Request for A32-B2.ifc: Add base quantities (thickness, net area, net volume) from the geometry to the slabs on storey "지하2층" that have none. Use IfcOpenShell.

First a look at what the model holds.

```python
import ifcopenshell
import ifcopenshell.util.element
import ifcopenshell.util.unit

model = ifcopenshell.open("A32-B2.ifc")
print(model.schema)
for unit_type in ("LENGTHUNIT", "AREAUNIT", "VOLUMEUNIT"):
    print(unit_type, ifcopenshell.util.unit.calculate_unit_scale(model, unit_type))
storey = next(s for s in model.by_type("IfcBuildingStorey") if s.Name == "지하2층")
slabs = [e for e in ifcopenshell.util.element.get_decomposition(storey) if e.is_a("IfcSlab")]
for e in sorted(slabs, key=lambda e: e.id()):
    print(e.id(), e.is_a(), e.Name, list(ifcopenshell.util.element.get_psets(e, qtos_only=True)), sep=" | ")
```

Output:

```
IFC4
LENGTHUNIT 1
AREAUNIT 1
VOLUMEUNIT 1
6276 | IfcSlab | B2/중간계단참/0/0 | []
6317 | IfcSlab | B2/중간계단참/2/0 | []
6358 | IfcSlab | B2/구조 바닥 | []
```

```python
import ifcopenshell
import ifcopenshell.api.pset
import ifcopenshell.geom
import ifcopenshell.util.element
import ifcopenshell.util.shape
import ifcopenshell.util.unit

model = ifcopenshell.open("A32-B2.ifc")
unit_scale = ifcopenshell.util.unit.calculate_unit_scale(model)
area_scale = ifcopenshell.util.unit.calculate_unit_scale(model, "AREAUNIT")
volume_scale = ifcopenshell.util.unit.calculate_unit_scale(model, "VOLUMEUNIT")
settings = ifcopenshell.geom.settings()

storey = next(s for s in model.by_type("IfcBuildingStorey") if s.Name == "지하2층")
slabs = [e for e in ifcopenshell.util.element.get_decomposition(storey) if e.is_a("IfcSlab")]

for e in sorted(slabs, key=lambda e: e.id()):
    if ifcopenshell.util.element.get_psets(e, qtos_only=True, should_inherit=False):
        continue
    # Geometry comes back in metres, in the element's own axes.
    shape = ifcopenshell.geom.create_shape(settings, e)
    values = {
        "Width": ifcopenshell.util.shape.get_z(shape.geometry) / unit_scale,
        "NetArea": ifcopenshell.util.shape.get_footprint_area(shape.geometry) / area_scale,
        "NetVolume": ifcopenshell.util.shape.get_volume(shape.geometry) / volume_scale,
    }
    qto = ifcopenshell.api.pset.add_qto(model, product=e, name="Qto_SlabBaseQuantities")
    ifcopenshell.api.pset.edit_qto(model, qto=qto, properties=values)
    print(e.id(), {k: round(v, 3) for k, v in values.items()})

model.write("A32-B2_edited.ifc")
```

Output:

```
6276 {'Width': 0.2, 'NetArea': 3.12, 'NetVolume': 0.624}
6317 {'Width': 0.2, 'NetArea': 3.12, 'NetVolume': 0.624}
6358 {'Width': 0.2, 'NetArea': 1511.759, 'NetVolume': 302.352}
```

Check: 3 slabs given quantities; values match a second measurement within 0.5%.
